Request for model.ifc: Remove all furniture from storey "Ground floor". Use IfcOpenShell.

First a look at what the model holds.

```python
import ifcopenshell
import ifcopenshell.util.element

model = ifcopenshell.open("model.ifc")
print(model.schema)
storey = next(s for s in model.by_type("IfcBuildingStorey") if s.Name == "Ground floor")
furniture = [e for e in ifcopenshell.util.element.get_decomposition(storey) if e.is_a("IfcFurnishingElement")]
seen = {}
for e in furniture:
    element_type = ifcopenshell.util.element.get_type(e)
    name = element_type.Name if element_type not in (None, e) else None
    seen[name] = seen.get(name, 0) + 1
for name, count in sorted(seen.items(), key=str):
    print(count, "x", name)
```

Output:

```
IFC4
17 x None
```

```python
import ifcopenshell
import ifcopenshell.api.root
import ifcopenshell.util.element

model = ifcopenshell.open("model.ifc")

storey = next(s for s in model.by_type("IfcBuildingStorey") if s.Name == "Ground floor")
furniture = [e for e in ifcopenshell.util.element.get_decomposition(storey) if e.is_a("IfcFurnishingElement")]

for e in furniture:
    ifcopenshell.api.root.remove_product(model, product=e)
print(len(furniture), "removed")

model.write("model_rev.ifc")
```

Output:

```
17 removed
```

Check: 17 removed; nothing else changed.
